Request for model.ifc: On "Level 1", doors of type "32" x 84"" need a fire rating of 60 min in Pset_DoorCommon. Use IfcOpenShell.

First a look at what the model holds.

```python
import ifcopenshell
import ifcopenshell.util.element

model = ifcopenshell.open("model.ifc")
print(model.schema)
storey = next(s for s in model.by_type("IfcBuildingStorey") if s.Name == "Level 1")
doors = [e for e in ifcopenshell.util.element.get_decomposition(storey) if e.is_a("IfcDoor")]
seen = {}
for e in doors:
    element_type = ifcopenshell.util.element.get_type(e)
    key = (element_type.Name if element_type != e and element_type else None, ifcopenshell.util.element.get_pset(e, "Pset_DoorCommon", "FireRating"))
    seen[key] = seen.get(key, 0) + 1
for (name, value), count in sorted(seen.items(), key=str):
    print(count, "x", name, "|", value)
```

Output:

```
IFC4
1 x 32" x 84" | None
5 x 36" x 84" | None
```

```python
import ifcopenshell
import ifcopenshell.api.pset
import ifcopenshell.util.element

model = ifcopenshell.open("model.ifc")

storey = next(s for s in model.by_type("IfcBuildingStorey") if s.Name == "Level 1")
doors = [e for e in ifcopenshell.util.element.get_decomposition(storey) if e.is_a("IfcDoor")]

count = 0
for e in doors:
    element_type = ifcopenshell.util.element.get_type(e)
    if element_type in (None, e) or element_type.Name != '32" x 84"':
        continue
    # add_pset returns the element's existing set when there is one.
    pset = ifcopenshell.api.pset.add_pset(model, product=e, name="Pset_DoorCommon")
    ifcopenshell.api.pset.edit_pset(model, pset=pset, properties={"FireRating": "60 min"})
    count += 1

print(count, "doors updated")

model.write("model_v2.ifc")
```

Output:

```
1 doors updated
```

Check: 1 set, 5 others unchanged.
